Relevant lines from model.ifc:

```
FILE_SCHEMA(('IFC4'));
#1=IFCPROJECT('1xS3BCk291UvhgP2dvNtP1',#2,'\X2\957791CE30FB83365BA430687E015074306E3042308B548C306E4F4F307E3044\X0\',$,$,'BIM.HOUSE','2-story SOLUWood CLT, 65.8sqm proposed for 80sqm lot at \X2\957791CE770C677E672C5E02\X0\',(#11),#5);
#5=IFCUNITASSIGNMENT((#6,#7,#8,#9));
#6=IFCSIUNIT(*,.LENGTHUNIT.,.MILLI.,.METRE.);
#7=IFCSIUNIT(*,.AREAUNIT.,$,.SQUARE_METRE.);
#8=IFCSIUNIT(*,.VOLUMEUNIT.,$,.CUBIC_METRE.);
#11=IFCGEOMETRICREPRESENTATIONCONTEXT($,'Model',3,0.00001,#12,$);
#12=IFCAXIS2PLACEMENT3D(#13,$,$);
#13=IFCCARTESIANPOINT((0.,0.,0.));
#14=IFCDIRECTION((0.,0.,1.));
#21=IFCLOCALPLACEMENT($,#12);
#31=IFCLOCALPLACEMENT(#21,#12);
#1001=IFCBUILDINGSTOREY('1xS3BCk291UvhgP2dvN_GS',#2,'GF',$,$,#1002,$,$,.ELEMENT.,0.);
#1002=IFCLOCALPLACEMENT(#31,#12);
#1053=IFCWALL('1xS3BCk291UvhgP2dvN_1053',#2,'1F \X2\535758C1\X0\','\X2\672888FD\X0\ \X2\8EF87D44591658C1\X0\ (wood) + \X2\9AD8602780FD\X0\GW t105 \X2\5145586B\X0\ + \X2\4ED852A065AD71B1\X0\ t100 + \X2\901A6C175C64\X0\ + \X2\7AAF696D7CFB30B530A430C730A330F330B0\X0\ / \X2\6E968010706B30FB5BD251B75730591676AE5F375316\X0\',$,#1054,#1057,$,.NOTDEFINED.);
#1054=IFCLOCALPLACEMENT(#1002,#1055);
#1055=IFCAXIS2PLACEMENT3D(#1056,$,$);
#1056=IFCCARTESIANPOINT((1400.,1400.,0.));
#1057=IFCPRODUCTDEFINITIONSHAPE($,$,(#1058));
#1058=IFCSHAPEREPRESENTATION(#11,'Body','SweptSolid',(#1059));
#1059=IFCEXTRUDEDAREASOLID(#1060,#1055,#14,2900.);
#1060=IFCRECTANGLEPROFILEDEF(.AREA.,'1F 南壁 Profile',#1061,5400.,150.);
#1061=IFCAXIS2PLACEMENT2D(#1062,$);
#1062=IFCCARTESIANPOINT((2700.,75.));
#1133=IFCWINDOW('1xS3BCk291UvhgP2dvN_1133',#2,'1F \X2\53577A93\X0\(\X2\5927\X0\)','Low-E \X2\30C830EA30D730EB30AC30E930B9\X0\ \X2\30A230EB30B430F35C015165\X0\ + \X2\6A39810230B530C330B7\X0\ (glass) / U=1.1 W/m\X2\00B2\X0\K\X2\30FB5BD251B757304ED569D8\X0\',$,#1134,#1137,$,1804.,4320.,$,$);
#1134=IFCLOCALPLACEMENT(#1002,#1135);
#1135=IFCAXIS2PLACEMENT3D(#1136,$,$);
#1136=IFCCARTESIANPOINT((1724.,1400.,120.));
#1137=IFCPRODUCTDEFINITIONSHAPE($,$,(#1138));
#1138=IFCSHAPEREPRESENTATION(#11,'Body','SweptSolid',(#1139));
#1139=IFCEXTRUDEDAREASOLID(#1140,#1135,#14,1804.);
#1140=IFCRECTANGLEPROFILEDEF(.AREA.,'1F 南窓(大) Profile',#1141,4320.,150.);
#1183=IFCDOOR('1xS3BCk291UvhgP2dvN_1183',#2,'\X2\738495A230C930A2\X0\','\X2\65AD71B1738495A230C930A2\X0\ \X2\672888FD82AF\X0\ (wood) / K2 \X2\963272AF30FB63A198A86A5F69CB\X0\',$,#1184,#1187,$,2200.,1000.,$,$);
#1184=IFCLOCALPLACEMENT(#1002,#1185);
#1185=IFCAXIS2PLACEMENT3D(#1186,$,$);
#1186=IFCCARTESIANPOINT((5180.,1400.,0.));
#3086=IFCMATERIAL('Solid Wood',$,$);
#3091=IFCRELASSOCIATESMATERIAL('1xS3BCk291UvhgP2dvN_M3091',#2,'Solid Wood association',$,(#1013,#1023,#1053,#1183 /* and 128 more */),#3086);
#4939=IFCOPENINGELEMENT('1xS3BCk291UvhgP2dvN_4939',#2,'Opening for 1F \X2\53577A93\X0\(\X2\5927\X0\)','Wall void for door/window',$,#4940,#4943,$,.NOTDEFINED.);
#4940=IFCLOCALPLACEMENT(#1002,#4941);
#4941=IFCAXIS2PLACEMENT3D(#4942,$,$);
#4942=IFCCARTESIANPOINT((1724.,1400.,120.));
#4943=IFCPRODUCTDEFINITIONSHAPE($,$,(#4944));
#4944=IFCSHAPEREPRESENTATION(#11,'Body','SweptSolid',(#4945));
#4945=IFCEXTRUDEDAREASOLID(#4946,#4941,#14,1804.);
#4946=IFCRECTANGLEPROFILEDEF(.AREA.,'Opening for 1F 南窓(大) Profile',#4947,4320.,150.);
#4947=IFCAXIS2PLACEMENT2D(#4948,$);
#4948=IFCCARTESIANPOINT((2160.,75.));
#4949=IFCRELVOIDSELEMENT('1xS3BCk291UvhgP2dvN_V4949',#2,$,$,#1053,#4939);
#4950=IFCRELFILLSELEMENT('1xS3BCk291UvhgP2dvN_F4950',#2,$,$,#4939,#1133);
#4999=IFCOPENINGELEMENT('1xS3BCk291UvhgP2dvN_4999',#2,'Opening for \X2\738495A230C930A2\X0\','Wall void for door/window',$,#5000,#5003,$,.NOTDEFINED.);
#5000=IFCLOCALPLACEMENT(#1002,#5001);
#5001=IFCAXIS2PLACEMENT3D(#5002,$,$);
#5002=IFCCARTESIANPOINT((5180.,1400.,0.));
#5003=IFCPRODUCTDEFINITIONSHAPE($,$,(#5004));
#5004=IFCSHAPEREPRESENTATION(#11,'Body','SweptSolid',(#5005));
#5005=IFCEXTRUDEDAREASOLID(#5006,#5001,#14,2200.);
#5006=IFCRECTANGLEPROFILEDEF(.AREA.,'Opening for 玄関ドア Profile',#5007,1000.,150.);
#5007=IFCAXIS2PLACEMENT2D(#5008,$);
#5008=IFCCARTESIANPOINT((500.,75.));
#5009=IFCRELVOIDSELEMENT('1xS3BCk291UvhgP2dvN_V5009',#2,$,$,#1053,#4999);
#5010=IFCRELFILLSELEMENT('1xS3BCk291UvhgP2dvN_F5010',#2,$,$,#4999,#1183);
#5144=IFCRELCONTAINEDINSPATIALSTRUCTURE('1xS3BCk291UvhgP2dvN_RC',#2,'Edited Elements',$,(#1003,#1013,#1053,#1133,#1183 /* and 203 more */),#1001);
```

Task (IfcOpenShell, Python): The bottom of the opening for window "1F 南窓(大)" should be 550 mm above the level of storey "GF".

```python
import numpy as np
import ifcopenshell
import ifcopenshell.api.geometry
import ifcopenshell.geom
import ifcopenshell.util.element
import ifcopenshell.util.placement
import ifcopenshell.util.shape
import ifcopenshell.util.unit

model = ifcopenshell.open("model.ifc")
unit_scale = ifcopenshell.util.unit.calculate_unit_scale(model)

window = model.by_guid("1xS3BCk291UvhgP2dvN_1133")
opening = window.FillsVoids[0].RelatingOpeningElement
storey = ifcopenshell.util.element.get_container(window, ifc_class="IfcBuildingStorey")
level = ifcopenshell.util.placement.get_local_placement(storey.ObjectPlacement)[2, 3]

# The opening's origin need not be at the sill, so measure its lowest point.
shape = ifcopenshell.geom.create_shape(ifcopenshell.geom.settings(), opening)
bottom = ifcopenshell.util.shape.get_shape_bottom_elevation(shape, shape.geometry) / unit_scale
dz = level + 550.0 - bottom

shift = np.array([0.0, 0.0, dz])
# The window is not placed relative to its opening, so move both.
for product in (opening, window):
    matrix = ifcopenshell.util.placement.get_local_placement(product.ObjectPlacement)
    matrix[:3, 3] += shift
    ifcopenshell.api.geometry.edit_object_placement(model, product=product, matrix=matrix, is_si=False)

print(f"moved by {dz * unit_scale:+.3f} m")

model.write("model_updated.ifc")
```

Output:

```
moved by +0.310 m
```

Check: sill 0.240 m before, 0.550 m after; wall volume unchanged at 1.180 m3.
